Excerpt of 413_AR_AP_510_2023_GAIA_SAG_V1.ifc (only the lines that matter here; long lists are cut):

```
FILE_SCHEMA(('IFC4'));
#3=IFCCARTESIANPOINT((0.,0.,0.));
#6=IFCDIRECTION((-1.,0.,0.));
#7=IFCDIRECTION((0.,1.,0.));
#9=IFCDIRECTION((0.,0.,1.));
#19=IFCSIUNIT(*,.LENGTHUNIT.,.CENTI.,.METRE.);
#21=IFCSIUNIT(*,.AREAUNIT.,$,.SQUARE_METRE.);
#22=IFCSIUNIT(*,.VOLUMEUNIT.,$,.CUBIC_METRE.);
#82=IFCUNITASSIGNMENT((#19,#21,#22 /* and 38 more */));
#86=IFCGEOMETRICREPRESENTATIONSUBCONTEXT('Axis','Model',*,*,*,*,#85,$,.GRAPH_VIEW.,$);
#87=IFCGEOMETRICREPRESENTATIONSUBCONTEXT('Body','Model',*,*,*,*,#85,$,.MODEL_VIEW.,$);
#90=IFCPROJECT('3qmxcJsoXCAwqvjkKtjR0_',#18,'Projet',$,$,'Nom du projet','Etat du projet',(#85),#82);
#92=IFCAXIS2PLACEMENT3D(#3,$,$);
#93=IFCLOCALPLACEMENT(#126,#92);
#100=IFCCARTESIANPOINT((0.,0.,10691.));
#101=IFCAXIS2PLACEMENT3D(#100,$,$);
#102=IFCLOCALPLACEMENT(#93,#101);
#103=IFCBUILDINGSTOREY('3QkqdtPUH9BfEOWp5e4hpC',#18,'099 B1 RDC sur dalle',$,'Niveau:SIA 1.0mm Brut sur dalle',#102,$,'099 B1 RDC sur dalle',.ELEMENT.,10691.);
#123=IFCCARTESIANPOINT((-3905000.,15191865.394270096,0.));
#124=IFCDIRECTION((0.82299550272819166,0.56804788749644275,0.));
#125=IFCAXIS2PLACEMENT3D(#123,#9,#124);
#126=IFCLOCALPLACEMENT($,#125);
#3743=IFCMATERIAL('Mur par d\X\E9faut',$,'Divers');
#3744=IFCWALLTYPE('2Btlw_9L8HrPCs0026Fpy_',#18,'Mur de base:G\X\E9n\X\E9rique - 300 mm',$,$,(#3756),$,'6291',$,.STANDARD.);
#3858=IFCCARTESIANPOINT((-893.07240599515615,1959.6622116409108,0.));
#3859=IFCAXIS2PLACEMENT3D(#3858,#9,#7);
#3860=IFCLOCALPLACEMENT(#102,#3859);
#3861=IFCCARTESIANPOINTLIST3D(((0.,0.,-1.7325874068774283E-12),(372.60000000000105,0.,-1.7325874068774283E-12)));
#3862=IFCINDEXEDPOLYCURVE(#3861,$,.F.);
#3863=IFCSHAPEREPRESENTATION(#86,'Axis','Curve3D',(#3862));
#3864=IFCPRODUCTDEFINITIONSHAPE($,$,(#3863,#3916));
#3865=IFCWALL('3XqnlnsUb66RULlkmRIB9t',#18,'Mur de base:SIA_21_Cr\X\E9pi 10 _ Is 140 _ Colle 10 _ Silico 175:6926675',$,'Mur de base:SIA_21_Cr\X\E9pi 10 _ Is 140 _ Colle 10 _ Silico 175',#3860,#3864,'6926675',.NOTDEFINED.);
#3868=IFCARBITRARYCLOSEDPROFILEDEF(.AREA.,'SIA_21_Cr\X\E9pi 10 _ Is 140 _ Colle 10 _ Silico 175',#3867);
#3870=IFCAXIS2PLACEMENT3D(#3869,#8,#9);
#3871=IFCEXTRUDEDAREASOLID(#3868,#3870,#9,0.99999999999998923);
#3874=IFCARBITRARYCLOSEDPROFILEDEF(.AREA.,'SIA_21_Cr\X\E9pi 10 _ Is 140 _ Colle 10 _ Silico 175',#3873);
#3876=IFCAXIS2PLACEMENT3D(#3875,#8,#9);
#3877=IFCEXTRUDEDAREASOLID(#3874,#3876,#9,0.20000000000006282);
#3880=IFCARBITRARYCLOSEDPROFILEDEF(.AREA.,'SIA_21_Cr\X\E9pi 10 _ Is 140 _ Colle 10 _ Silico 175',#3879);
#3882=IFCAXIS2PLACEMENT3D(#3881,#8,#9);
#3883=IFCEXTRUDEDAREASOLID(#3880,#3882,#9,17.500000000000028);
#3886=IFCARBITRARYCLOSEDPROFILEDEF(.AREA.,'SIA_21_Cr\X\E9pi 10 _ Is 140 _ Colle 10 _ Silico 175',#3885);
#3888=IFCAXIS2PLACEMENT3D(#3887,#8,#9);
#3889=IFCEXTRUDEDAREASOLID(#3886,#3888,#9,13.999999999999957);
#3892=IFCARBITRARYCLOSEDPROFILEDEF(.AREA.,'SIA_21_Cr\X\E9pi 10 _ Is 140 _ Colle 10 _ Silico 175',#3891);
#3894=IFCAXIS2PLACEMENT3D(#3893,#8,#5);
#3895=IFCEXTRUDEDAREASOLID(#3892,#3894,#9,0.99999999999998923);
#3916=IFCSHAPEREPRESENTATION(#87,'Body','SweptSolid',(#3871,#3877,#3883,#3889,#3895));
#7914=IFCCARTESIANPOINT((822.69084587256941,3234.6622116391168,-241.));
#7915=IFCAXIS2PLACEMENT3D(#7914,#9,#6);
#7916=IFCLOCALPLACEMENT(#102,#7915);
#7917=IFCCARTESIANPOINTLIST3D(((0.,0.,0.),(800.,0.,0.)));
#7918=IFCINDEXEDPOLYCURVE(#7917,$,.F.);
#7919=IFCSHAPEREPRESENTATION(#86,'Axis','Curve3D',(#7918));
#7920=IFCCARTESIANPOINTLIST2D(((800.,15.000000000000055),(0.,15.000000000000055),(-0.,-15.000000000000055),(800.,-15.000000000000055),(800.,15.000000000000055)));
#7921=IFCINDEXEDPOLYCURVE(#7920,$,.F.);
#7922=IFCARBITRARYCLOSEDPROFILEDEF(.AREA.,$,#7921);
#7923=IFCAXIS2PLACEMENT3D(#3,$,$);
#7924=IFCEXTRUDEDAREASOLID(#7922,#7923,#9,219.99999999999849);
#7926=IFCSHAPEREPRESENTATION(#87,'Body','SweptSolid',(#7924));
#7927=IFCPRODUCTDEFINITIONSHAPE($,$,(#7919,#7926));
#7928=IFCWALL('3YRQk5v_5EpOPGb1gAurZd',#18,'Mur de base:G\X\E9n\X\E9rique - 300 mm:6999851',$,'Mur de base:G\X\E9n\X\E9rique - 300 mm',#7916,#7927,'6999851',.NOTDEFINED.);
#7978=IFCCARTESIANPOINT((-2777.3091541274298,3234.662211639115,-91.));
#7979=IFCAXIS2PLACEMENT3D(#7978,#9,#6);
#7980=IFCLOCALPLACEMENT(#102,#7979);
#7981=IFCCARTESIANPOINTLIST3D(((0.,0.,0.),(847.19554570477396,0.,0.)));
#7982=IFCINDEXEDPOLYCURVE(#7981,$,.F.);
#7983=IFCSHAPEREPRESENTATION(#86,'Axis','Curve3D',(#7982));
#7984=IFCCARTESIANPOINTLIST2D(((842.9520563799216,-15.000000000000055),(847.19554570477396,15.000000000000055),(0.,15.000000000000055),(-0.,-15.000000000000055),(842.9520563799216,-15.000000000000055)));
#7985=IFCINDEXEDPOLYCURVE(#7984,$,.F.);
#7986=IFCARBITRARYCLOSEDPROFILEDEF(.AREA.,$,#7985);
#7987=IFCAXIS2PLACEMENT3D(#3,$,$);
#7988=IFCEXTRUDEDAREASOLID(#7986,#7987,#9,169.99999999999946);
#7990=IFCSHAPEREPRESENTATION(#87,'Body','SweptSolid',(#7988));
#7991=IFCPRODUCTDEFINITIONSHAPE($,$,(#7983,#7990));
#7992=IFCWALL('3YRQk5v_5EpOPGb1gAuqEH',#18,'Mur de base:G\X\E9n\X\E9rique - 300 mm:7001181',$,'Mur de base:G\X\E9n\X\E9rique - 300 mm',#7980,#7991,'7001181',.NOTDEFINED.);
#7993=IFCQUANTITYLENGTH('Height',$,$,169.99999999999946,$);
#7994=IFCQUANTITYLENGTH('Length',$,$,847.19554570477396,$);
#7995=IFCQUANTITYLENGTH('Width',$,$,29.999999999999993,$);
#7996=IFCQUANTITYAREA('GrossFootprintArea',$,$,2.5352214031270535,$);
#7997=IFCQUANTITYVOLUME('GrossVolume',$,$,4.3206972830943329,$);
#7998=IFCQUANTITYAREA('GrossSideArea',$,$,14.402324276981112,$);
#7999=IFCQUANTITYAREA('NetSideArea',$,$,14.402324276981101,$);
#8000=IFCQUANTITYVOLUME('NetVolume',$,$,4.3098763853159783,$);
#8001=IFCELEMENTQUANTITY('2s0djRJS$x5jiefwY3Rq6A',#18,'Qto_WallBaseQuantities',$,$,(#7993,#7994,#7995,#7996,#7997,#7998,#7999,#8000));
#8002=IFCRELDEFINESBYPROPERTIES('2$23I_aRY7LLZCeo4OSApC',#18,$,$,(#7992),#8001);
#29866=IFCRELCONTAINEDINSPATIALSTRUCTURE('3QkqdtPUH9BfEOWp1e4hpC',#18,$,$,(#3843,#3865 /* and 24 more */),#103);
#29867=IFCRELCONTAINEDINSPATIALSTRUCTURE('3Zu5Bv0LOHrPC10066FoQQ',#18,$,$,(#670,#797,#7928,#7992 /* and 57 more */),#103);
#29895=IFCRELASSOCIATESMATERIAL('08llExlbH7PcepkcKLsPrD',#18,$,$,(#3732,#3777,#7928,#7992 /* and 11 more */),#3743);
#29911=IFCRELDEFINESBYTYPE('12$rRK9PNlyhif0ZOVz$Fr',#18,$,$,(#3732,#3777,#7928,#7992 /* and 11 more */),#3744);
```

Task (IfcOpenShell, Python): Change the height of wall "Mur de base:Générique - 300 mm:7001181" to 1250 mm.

```python
import ifcopenshell
import ifcopenshell.api.pset
import ifcopenshell.geom
import ifcopenshell.util.element
import ifcopenshell.util.representation
import ifcopenshell.util.shape
import ifcopenshell.util.unit

model = ifcopenshell.open("413_AR_AP_510_2023_GAIA_SAG_V1.ifc")
unit_scale = ifcopenshell.util.unit.calculate_unit_scale(model)
area_scale = ifcopenshell.util.unit.calculate_unit_scale(model, "AREAUNIT")
volume_scale = ifcopenshell.util.unit.calculate_unit_scale(model, "VOLUMEUNIT")
settings = ifcopenshell.geom.settings()


def volume(element):
    """Net volume in cubic metres, openings subtracted."""
    shape = ifcopenshell.geom.create_shape(settings, element)
    return ifcopenshell.util.shape.get_volume(shape.geometry)


wall = model.by_id(7992)
before = volume(wall)

body = ifcopenshell.util.representation.get_representation(wall, "Model", "Body")
solid = body.Items[0]
old_height = solid.Depth
solid.Depth = 1.25 / unit_scale
after = volume(wall)
thickness = 0.3  # wall thickness in metres

# Update the stored height, areas and volumes.
qto = model.by_id(ifcopenshell.util.element.get_pset(wall, "Qto_WallBaseQuantities", should_inherit=False)["id"])
ifcopenshell.api.pset.edit_qto(model, qto=qto, properties={
    "Height": solid.Depth,
    "GrossVolume": ifcopenshell.util.element.get_pset(wall, "Qto_WallBaseQuantities", "GrossVolume") * solid.Depth / old_height,
    "GrossSideArea": ifcopenshell.util.element.get_pset(wall, "Qto_WallBaseQuantities", "GrossSideArea") * solid.Depth / old_height,
    "NetSideArea": after / thickness / area_scale,
    "NetVolume": after / volume_scale,
})

print(f"height {old_height:g} -> {solid.Depth:g}, volume {before:.3f} -> {after:.3f} m3")

model.write("413_AR_AP_510_2023_GAIA_SAG_V1_edited.ifc")
```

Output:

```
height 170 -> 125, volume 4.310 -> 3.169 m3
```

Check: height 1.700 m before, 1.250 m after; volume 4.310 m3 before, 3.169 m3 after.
